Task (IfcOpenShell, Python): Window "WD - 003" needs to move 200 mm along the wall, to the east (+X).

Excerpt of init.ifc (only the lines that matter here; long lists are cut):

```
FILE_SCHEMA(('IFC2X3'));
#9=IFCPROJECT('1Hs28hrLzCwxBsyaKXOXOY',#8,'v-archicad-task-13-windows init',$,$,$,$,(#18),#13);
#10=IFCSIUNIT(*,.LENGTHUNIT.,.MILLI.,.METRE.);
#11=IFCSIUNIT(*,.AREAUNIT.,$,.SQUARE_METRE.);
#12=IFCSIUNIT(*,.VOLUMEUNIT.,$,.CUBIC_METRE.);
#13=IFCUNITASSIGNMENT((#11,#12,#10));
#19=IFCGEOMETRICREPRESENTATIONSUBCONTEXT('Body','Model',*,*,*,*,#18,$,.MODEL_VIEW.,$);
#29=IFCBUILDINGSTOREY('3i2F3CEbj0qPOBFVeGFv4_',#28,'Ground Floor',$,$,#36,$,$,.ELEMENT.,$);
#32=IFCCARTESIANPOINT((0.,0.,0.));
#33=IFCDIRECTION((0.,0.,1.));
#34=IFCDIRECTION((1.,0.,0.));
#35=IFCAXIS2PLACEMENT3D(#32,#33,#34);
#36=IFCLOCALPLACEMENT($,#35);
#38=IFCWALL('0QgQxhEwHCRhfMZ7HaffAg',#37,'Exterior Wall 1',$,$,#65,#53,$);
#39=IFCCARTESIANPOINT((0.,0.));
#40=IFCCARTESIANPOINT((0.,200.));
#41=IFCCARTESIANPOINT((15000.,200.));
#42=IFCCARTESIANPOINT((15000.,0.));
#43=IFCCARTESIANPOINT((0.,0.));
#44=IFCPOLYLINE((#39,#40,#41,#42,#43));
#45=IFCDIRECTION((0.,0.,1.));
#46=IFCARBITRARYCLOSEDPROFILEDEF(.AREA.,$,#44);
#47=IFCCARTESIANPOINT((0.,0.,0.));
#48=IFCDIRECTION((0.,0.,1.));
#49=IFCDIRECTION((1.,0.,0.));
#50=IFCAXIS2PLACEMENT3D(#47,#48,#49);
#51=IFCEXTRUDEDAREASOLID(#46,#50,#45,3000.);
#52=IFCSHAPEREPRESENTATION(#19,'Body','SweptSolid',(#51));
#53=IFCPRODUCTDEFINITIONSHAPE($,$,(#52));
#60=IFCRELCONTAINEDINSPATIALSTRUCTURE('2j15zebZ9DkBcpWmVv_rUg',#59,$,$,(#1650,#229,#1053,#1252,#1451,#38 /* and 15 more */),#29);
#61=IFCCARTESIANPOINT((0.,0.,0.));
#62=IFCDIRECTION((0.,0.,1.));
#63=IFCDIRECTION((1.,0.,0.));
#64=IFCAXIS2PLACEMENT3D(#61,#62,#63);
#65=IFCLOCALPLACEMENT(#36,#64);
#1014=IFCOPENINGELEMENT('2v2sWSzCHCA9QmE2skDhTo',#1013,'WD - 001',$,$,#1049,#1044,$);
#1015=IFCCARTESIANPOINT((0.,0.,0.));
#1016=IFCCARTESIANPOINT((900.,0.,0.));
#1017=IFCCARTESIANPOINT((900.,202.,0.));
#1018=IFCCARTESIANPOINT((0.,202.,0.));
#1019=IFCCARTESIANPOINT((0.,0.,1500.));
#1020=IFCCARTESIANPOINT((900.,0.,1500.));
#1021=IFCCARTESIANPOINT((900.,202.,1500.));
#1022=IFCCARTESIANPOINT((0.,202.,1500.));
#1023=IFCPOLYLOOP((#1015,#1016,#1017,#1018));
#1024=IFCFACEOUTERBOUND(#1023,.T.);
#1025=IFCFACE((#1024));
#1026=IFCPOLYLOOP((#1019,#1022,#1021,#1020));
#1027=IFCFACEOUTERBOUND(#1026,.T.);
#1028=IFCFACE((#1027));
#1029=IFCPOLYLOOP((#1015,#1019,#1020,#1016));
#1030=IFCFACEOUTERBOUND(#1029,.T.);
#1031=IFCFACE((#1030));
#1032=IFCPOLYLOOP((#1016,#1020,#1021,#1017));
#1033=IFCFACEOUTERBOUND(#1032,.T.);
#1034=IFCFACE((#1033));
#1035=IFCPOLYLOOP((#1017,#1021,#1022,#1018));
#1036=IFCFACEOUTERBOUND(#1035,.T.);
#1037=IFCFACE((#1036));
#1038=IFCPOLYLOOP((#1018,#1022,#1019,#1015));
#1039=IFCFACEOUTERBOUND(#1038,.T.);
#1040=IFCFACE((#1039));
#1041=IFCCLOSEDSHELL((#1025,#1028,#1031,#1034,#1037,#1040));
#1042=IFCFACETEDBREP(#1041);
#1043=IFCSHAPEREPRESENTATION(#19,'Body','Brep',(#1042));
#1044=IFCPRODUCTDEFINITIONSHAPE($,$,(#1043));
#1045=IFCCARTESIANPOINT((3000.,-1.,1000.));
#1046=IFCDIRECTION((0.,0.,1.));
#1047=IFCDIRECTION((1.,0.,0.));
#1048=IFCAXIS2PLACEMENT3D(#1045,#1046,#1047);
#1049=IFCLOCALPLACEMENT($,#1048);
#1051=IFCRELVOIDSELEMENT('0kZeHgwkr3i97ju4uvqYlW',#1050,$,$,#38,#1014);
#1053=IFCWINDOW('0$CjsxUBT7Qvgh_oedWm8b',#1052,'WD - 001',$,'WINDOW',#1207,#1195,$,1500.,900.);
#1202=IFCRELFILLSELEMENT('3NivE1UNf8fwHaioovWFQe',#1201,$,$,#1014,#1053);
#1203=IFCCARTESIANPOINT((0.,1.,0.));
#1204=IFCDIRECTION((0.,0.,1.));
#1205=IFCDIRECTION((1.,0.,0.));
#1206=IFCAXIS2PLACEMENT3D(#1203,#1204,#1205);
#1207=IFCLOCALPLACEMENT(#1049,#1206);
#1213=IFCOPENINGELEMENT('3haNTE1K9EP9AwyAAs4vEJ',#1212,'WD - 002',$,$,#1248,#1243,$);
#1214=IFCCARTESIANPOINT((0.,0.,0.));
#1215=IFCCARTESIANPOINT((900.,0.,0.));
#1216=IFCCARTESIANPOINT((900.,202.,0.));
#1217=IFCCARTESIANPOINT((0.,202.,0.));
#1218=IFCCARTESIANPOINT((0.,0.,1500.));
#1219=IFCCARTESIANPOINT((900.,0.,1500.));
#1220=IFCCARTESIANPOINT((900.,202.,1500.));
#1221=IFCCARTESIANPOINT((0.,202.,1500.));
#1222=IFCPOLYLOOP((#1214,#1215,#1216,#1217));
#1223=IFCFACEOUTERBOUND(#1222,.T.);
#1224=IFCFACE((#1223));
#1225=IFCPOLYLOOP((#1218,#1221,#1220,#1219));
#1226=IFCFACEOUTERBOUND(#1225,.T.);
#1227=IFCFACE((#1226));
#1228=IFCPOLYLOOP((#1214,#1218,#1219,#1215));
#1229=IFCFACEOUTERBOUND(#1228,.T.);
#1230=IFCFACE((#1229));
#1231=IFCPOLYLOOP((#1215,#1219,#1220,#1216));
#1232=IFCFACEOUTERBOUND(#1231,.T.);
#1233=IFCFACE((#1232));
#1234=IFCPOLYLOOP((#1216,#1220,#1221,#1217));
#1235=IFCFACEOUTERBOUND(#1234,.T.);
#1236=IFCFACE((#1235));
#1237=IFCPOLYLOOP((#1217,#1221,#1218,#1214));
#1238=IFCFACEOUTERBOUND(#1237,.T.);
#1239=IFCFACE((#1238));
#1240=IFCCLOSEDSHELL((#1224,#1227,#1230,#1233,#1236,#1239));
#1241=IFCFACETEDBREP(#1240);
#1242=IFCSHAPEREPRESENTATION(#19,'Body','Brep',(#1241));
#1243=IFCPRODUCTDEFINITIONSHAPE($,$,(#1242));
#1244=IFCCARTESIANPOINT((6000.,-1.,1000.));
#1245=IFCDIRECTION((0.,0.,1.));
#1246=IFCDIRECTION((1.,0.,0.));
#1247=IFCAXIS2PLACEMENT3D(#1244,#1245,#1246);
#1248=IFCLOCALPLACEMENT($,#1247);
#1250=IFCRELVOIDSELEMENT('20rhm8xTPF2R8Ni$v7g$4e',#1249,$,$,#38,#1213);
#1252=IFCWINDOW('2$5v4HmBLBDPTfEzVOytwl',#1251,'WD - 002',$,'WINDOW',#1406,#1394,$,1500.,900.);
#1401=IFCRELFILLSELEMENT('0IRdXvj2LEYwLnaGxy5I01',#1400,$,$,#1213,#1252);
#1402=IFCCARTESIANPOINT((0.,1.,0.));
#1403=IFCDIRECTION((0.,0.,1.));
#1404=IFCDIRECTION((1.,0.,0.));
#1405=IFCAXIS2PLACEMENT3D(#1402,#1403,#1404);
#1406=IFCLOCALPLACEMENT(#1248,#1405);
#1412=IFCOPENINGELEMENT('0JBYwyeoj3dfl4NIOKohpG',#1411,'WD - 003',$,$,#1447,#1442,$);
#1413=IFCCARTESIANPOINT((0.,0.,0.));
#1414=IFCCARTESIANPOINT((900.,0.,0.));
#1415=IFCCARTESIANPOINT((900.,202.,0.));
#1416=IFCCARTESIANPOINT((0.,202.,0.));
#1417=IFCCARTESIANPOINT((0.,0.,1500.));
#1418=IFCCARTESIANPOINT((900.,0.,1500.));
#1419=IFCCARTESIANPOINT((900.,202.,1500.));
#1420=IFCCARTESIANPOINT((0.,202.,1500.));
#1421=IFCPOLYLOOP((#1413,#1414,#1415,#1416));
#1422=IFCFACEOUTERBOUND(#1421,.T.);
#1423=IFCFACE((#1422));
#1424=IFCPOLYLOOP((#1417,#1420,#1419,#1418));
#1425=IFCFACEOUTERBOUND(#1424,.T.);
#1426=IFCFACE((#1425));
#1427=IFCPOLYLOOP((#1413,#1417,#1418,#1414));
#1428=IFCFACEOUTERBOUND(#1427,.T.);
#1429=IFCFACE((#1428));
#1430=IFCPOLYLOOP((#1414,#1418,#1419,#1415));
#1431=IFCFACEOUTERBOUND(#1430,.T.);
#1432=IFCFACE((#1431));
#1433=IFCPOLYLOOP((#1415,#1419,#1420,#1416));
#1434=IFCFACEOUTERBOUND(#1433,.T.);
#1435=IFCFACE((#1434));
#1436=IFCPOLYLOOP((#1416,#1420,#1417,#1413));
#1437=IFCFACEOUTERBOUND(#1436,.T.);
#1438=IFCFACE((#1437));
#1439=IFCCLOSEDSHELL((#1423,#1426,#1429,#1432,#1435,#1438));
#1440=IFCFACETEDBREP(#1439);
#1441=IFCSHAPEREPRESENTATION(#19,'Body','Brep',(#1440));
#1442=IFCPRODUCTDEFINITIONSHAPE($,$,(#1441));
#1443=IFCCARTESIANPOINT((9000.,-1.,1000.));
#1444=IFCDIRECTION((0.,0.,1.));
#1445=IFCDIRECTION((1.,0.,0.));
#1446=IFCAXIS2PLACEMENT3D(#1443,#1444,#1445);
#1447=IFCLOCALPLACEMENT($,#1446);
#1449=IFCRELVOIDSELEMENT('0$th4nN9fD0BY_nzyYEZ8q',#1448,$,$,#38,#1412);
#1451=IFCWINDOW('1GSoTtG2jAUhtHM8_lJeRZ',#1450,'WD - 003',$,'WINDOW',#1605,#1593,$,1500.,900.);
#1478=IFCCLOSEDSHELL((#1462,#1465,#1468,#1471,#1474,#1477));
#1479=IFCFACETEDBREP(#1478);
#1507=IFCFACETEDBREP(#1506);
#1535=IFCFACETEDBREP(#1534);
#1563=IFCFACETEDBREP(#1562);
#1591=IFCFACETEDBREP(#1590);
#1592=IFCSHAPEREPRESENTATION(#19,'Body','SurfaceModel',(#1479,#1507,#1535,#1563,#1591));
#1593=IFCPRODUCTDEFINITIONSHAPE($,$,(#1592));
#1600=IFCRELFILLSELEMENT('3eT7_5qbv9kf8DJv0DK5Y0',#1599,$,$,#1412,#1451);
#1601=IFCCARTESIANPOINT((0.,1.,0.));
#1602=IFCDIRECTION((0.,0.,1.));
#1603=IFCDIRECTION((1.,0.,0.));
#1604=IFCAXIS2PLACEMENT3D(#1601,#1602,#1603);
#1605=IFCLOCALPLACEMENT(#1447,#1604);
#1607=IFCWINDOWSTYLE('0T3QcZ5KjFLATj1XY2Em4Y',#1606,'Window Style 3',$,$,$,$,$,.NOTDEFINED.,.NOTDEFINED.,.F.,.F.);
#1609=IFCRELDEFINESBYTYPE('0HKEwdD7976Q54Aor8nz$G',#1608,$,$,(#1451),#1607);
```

```python
import ifcopenshell
import ifcopenshell.api.geometry
import ifcopenshell.util.placement
import ifcopenshell.util.unit

model = ifcopenshell.open("init.ifc")
unit_scale = ifcopenshell.util.unit.calculate_unit_scale(model)

window = model.by_id(1451)
opening = window.FillsVoids[0].RelatingOpeningElement
wall = opening.VoidsElements[0].RelatingBuildingElement

wall_matrix = ifcopenshell.util.placement.get_local_placement(wall.ObjectPlacement)
shift = wall_matrix[:3, 0] * 0.2 / unit_scale
before = ifcopenshell.util.placement.get_local_placement(window.ObjectPlacement)[:3, 3].copy()

# The window is placed relative to its opening, so it follows when the opening moves.
matrix = ifcopenshell.util.placement.get_local_placement(opening.ObjectPlacement)
matrix[:3, 3] += shift
ifcopenshell.api.geometry.edit_object_placement(
    model, product=opening, matrix=matrix, is_si=False, should_transform_children=True
)

after = ifcopenshell.util.placement.get_local_placement(window.ObjectPlacement)[:3, 3]
print("window moved by", (after - before).round(3) + 0.0)

model.write("init_edited.ifc")
```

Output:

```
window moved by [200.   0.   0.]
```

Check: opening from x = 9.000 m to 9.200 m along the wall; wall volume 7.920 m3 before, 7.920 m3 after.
